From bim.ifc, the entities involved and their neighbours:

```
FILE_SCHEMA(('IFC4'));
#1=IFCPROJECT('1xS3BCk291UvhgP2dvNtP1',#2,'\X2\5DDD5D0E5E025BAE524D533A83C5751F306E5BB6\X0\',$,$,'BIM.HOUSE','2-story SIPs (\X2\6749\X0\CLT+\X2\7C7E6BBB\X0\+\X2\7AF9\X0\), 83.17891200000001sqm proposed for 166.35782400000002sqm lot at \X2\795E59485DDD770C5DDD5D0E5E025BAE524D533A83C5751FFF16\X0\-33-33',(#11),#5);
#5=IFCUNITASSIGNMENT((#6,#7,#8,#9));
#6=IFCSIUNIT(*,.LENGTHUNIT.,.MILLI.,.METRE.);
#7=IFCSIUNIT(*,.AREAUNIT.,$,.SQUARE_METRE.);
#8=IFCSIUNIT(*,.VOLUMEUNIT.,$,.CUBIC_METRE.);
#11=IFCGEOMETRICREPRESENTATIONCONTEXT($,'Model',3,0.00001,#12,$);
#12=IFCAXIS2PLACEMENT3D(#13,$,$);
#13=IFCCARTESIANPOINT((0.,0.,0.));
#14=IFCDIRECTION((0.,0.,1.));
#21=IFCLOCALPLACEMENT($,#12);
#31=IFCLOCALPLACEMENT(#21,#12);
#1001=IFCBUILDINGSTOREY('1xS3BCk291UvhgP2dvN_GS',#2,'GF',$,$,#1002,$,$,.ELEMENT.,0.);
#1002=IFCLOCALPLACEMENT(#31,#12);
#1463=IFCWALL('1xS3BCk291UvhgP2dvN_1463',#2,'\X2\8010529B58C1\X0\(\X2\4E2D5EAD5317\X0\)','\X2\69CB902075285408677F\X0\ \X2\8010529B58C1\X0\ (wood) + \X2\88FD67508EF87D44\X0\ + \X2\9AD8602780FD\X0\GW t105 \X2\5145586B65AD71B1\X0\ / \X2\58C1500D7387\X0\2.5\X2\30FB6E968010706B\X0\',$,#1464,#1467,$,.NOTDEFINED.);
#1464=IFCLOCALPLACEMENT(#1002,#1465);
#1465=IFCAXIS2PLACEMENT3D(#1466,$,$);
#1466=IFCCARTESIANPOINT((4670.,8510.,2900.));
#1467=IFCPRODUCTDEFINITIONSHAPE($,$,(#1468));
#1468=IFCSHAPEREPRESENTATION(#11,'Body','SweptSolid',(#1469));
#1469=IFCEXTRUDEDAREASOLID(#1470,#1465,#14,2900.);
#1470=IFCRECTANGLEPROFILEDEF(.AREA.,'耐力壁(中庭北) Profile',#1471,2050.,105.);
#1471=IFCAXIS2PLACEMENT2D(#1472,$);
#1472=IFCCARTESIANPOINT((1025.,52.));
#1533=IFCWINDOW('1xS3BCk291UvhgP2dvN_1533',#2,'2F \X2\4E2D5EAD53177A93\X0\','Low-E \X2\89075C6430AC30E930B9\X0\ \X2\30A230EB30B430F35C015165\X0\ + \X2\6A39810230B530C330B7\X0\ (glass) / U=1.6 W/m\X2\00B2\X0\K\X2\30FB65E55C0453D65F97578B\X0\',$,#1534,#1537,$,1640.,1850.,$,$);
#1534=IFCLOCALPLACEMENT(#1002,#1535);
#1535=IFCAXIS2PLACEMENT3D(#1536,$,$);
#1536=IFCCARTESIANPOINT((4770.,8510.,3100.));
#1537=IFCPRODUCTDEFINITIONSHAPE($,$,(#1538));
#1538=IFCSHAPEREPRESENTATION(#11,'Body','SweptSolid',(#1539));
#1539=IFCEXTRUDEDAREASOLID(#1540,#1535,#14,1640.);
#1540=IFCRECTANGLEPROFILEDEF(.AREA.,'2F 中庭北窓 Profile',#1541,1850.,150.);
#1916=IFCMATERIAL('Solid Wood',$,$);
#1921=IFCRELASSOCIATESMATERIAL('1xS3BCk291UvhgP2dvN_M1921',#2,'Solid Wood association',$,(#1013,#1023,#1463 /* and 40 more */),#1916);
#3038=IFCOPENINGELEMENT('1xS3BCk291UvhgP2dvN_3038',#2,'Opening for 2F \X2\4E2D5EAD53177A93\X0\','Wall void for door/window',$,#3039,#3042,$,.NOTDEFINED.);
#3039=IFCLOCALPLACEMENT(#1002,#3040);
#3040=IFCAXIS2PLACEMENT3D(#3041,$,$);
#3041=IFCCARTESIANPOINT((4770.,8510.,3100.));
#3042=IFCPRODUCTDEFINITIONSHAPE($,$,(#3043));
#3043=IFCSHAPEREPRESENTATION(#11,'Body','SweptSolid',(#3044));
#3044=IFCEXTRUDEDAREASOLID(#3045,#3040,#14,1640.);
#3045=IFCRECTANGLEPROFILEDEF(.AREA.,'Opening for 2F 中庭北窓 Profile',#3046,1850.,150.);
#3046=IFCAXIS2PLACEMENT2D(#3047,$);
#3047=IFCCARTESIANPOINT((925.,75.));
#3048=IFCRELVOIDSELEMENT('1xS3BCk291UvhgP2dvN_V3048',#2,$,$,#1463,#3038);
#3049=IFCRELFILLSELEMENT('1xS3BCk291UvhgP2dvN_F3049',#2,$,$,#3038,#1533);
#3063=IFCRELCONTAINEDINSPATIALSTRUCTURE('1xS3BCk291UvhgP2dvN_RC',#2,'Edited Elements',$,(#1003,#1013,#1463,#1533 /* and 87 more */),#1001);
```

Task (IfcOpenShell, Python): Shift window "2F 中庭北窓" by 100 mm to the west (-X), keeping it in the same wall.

```python
import ifcopenshell
import ifcopenshell.api.geometry
import ifcopenshell.util.placement

model = ifcopenshell.open("bim.ifc")

window = model.by_id(1533)
opening = window.FillsVoids[0].RelatingOpeningElement
wall = opening.VoidsElements[0].RelatingBuildingElement

wall_matrix = ifcopenshell.util.placement.get_local_placement(wall.ObjectPlacement)
shift = wall_matrix[:3, 0] * -100.0
before = ifcopenshell.util.placement.get_local_placement(window.ObjectPlacement)[:3, 3].copy()

# The window is not placed relative to its opening, so move both.
for product in (opening, window):
    matrix = ifcopenshell.util.placement.get_local_placement(product.ObjectPlacement)
    matrix[:3, 3] += shift
    ifcopenshell.api.geometry.edit_object_placement(model, product=product, matrix=matrix, is_si=False)

after = ifcopenshell.util.placement.get_local_placement(window.ObjectPlacement)[:3, 3]
print("window moved by", (after - before).round(3) + 0.0)

model.write("bim_v2.ifc")
```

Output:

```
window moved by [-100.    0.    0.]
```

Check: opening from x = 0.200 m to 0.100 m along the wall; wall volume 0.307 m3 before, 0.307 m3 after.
